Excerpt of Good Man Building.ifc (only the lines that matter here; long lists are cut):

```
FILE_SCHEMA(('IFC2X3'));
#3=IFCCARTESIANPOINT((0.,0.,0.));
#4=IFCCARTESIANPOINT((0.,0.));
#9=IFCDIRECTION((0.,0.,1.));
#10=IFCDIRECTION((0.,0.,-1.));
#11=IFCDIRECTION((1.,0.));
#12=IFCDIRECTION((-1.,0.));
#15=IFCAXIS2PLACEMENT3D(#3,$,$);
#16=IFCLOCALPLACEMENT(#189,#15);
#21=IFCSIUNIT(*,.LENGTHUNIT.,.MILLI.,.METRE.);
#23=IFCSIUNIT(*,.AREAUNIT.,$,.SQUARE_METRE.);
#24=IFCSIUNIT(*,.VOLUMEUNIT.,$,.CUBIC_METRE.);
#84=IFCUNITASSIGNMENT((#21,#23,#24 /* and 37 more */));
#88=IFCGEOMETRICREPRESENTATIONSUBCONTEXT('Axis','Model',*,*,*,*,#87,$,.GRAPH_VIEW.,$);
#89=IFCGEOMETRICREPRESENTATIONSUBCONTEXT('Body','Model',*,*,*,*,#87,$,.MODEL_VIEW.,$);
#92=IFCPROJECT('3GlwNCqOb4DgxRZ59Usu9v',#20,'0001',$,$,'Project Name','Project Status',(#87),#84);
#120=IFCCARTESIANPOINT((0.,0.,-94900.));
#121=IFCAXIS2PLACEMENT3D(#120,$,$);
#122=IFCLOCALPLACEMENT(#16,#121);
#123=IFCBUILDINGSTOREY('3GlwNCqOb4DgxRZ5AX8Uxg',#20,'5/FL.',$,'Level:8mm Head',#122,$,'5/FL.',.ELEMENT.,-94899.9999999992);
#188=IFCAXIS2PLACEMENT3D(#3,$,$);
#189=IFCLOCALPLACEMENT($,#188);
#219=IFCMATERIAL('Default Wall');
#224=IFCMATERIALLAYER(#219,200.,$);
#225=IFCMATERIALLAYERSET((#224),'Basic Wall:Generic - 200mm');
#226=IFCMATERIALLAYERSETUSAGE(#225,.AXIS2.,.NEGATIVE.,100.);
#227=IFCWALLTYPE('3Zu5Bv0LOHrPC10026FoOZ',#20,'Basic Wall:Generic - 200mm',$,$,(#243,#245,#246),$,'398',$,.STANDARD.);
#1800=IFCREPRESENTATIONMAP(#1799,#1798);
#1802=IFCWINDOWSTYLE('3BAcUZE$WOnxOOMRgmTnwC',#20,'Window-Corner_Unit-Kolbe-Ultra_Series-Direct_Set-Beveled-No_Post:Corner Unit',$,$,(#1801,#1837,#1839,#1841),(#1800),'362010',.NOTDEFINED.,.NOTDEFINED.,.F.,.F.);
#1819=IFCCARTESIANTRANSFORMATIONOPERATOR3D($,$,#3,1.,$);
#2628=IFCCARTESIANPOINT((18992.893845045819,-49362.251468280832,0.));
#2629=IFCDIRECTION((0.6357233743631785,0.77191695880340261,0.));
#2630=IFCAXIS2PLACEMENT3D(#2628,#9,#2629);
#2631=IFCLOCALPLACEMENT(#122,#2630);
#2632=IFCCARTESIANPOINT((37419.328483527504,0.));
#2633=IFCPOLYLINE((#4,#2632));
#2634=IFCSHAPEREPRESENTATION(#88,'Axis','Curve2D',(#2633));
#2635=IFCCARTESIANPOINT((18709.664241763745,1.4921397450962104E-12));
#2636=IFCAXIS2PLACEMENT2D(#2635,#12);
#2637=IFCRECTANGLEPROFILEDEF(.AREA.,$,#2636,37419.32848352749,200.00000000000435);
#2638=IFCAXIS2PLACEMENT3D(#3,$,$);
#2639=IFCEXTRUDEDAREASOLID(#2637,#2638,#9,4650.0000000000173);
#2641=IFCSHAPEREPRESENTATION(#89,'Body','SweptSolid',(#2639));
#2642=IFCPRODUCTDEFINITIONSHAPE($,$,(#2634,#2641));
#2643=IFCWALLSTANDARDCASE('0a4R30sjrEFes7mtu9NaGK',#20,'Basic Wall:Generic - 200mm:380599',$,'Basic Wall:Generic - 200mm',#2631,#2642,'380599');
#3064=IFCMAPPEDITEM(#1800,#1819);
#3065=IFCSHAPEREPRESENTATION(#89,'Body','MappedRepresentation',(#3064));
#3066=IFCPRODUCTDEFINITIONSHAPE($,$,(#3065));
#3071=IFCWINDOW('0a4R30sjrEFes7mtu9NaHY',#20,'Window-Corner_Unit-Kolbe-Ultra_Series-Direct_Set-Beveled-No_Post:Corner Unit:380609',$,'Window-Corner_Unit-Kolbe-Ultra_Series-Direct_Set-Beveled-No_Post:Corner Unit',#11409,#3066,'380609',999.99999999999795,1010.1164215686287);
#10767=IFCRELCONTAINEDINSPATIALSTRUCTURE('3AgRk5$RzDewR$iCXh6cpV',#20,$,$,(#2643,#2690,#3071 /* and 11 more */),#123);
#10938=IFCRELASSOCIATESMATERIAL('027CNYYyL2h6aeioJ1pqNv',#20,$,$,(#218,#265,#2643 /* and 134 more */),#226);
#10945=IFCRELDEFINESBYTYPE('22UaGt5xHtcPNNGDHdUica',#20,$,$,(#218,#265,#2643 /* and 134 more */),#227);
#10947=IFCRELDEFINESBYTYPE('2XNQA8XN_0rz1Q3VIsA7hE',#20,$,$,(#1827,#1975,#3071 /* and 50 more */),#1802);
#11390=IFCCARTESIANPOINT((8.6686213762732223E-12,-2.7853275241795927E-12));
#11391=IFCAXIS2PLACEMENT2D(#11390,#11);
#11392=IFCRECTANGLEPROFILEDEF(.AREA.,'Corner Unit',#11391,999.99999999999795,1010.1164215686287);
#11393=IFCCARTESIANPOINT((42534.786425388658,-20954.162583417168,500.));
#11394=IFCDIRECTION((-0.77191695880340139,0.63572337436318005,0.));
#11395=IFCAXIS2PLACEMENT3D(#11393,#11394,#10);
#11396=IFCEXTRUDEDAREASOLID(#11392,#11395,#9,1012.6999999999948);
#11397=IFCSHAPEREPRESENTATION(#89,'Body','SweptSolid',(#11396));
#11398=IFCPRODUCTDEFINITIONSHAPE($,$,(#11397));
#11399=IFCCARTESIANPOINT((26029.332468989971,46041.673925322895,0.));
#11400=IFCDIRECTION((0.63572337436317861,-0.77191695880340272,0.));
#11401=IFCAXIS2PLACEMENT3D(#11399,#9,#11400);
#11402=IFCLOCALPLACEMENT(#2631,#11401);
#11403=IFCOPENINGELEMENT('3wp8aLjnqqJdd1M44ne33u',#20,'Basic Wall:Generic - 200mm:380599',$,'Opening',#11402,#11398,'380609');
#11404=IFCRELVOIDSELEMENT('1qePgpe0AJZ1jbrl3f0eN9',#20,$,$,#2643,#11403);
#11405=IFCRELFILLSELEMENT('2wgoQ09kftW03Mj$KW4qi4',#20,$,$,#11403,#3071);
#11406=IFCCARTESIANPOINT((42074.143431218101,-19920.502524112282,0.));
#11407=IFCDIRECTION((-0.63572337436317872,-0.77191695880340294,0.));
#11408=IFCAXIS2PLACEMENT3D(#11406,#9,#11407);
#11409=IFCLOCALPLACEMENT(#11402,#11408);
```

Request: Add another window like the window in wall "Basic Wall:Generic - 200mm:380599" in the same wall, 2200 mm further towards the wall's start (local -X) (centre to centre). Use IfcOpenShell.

```python
import ifcopenshell
import ifcopenshell.api.feature
import ifcopenshell.api.geometry
import ifcopenshell.api.root
import ifcopenshell.geom
import ifcopenshell.util.element
import ifcopenshell.util.placement
import ifcopenshell.util.shape
import ifcopenshell.util.unit

model = ifcopenshell.open("Good Man Building.ifc")
unit_scale = ifcopenshell.util.unit.calculate_unit_scale(model)
settings = ifcopenshell.geom.settings()


def volume(element):
    """Net volume in cubic metres, openings subtracted."""
    shape = ifcopenshell.geom.create_shape(settings, element)
    return ifcopenshell.util.shape.get_volume(shape.geometry)


def reuse_history(source, copy):
    """copy_class also copies each property set's owner history, people and application; keep the originals."""
    for rel in copy.IsDefinedBy:
        if rel.is_a("IfcRelDefinesByProperties") and (history := rel.RelatingPropertyDefinition.OwnerHistory):
            rel.RelatingPropertyDefinition.OwnerHistory = source.OwnerHistory
            ifcopenshell.util.element.remove_deep2(model, history)


window = model.by_guid("0a4R30sjrEFes7mtu9NaHY")
opening = window.FillsVoids[0].RelatingOpeningElement
wall = opening.VoidsElements[0].RelatingBuildingElement
before = volume(wall)
shift = ifcopenshell.util.placement.get_local_placement(wall.ObjectPlacement)[:3, 0] * -2.2 / unit_scale

# copy_class copies the void relationship, type, container and properties, but no geometry.
new_opening = ifcopenshell.api.root.copy_class(model, product=opening)
new_opening.Representation = ifcopenshell.util.element.copy_deep(
    model, opening.Representation, exclude=["IfcGeometricRepresentationContext", "IfcRepresentationMap"]
)
new_opening.Name = "Basic Wall:Generic - 200mm"
new_opening.Tag = None
new_window = ifcopenshell.api.root.copy_class(model, product=window)
new_window.Representation = ifcopenshell.util.element.copy_deep(
    model, window.Representation, exclude=["IfcGeometricRepresentationContext", "IfcRepresentationMap"]
)
new_window.Name = "Window-Corner_Unit-Kolbe-Ultra_Series-Direct_Set-Beveled-No_Post:Corner Unit"
new_window.Tag = None
reuse_history(window, new_window)
fills = ifcopenshell.api.feature.add_filling(model, opening=new_opening, element=new_window)
fills.OwnerHistory = new_window.OwnerHistory  # required in IFC2X3

for old, new in ((opening, new_opening), (window, new_window)):
    matrix = ifcopenshell.util.placement.get_local_placement(old.ObjectPlacement)
    matrix[:3, 3] += shift
    ifcopenshell.api.geometry.edit_object_placement(model, product=new, matrix=matrix, is_si=False)

after = volume(wall)

print(f"wall volume {before:.3f} -> {after:.3f} m3")

model.write("Good Man Building_updated.ifc")
```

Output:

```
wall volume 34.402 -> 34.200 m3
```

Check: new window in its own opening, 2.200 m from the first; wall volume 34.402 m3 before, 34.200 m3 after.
